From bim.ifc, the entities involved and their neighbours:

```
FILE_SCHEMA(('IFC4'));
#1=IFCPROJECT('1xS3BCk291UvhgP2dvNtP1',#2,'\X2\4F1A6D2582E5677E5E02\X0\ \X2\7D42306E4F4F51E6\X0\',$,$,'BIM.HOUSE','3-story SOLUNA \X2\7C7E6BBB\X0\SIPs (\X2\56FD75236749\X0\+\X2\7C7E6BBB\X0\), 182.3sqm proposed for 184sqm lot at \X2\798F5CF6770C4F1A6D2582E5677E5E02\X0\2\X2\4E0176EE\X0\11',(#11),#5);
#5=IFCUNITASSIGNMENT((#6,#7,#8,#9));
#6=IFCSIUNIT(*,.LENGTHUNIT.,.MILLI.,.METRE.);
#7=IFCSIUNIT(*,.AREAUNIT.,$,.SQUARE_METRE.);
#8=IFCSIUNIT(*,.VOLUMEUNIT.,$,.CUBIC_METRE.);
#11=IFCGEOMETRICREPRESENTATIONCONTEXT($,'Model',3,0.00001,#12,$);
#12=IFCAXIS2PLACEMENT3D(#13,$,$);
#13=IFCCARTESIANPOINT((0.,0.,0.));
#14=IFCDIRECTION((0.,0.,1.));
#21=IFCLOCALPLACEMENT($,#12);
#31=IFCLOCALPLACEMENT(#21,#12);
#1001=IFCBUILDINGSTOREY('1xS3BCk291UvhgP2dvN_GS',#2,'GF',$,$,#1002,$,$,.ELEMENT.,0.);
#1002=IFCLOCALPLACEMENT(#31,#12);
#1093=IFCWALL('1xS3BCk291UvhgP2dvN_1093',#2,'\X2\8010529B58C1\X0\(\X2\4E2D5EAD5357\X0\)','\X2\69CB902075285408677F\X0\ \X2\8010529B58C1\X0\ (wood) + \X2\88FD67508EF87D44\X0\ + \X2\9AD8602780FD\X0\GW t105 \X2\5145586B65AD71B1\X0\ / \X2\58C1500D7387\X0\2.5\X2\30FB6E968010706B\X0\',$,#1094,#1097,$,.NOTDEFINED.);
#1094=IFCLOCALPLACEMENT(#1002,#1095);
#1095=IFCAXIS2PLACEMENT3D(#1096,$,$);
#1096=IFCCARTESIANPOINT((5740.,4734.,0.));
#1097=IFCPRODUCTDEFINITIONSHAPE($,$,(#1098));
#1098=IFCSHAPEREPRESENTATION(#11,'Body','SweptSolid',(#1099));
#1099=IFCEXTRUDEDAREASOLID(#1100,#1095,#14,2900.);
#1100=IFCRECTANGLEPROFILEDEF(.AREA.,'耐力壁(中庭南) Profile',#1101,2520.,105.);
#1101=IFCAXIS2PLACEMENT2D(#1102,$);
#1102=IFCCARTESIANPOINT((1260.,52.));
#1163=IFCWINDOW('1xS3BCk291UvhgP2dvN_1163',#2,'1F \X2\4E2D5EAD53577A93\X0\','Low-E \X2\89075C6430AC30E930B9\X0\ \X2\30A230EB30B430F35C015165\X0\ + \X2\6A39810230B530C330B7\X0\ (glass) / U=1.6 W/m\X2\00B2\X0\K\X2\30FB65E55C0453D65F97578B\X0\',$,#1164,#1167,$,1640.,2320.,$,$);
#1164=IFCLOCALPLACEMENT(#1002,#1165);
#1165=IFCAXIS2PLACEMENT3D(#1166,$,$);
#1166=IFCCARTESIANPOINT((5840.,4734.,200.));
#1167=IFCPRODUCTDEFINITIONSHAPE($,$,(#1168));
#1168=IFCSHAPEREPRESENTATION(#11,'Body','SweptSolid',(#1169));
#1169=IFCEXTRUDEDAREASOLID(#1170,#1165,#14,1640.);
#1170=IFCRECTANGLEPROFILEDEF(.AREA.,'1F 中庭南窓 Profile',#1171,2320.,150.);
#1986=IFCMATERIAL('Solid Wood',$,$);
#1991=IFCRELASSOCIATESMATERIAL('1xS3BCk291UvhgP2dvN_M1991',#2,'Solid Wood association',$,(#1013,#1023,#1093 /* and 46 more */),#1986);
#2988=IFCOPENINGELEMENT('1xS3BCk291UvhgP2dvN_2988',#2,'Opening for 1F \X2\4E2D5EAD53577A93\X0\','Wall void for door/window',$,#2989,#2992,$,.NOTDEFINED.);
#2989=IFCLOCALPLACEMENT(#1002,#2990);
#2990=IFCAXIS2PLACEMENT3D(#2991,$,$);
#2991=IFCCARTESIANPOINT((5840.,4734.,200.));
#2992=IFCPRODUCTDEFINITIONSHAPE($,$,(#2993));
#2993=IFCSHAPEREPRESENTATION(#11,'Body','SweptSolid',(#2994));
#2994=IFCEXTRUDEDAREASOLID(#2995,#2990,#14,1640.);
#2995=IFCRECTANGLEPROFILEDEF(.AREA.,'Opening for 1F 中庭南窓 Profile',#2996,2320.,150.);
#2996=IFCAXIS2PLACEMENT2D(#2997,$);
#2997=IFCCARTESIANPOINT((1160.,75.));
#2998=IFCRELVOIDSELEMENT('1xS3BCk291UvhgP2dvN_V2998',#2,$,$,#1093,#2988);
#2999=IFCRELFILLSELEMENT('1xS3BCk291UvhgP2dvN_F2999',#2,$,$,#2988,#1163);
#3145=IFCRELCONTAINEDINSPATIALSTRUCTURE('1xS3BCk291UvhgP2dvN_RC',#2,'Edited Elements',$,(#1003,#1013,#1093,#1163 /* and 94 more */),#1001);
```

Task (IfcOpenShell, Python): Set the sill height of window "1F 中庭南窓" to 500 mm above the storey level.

```python
import numpy as np
import ifcopenshell
import ifcopenshell.api.geometry
import ifcopenshell.geom
import ifcopenshell.util.element
import ifcopenshell.util.placement
import ifcopenshell.util.shape
import ifcopenshell.util.unit

model = ifcopenshell.open("bim.ifc")
unit_scale = ifcopenshell.util.unit.calculate_unit_scale(model)

window = model.by_id(1163)
opening = window.FillsVoids[0].RelatingOpeningElement
storey = ifcopenshell.util.element.get_container(window, ifc_class="IfcBuildingStorey")
level = ifcopenshell.util.placement.get_local_placement(storey.ObjectPlacement)[2, 3]

# The opening's origin need not be at the sill, so measure its lowest point.
shape = ifcopenshell.geom.create_shape(ifcopenshell.geom.settings(), opening)
bottom = ifcopenshell.util.shape.get_shape_bottom_elevation(shape, shape.geometry) / unit_scale
dz = level + 0.5 / unit_scale - bottom

shift = np.array([0.0, 0.0, dz])
# The window is not placed relative to its opening, so move both.
for product in (opening, window):
    matrix = ifcopenshell.util.placement.get_local_placement(product.ObjectPlacement)
    matrix[:3, 3] += shift
    ifcopenshell.api.geometry.edit_object_placement(model, product=product, matrix=matrix, is_si=False)

print(f"moved by {dz * unit_scale:+.3f} m")

model.write("bim_rev.ifc")
```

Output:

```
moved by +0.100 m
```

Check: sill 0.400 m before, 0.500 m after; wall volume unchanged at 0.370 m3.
